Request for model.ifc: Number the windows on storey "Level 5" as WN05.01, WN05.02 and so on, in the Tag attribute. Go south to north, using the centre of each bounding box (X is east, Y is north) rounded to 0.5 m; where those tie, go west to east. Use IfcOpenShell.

First a look at what the model holds.

```python
import ifcopenshell
import ifcopenshell.util.element
import ifcopenshell.util.placement

model = ifcopenshell.open("model.ifc")
print(model.schema)
storey = next(s for s in model.by_type("IfcBuildingStorey") if s.Name == "Level 5")
windows = [e for e in ifcopenshell.util.element.get_decomposition(storey) if e.is_a("IfcWindow")]
for e in sorted(windows, key=lambda e: e.id()):
    origin = ifcopenshell.util.placement.get_local_placement(e.ObjectPlacement)[:3, 3]
    print(e.id(), e.Tag, e.Name, origin.round(2) + 0.0, sep=" | ")
```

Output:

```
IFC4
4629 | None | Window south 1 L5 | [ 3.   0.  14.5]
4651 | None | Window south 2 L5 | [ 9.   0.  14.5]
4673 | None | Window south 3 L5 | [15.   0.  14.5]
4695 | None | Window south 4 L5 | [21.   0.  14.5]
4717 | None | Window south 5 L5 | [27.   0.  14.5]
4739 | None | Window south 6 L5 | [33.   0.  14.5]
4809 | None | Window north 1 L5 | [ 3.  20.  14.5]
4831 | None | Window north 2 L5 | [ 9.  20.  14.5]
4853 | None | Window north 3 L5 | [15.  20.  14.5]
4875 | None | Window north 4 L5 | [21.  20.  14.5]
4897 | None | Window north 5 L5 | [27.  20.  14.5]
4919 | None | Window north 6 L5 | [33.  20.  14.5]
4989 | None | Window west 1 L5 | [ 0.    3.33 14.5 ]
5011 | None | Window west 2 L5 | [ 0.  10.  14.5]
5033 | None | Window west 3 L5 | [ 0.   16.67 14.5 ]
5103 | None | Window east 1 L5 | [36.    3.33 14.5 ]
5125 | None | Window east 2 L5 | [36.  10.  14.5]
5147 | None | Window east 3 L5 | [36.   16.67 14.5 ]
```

```python
import ifcopenshell
import ifcopenshell.geom
import ifcopenshell.util.element
import ifcopenshell.util.shape

model = ifcopenshell.open("model.ifc")
settings = ifcopenshell.geom.settings()
settings.set("use-world-coords", True)


def centre(element):
    shape = ifcopenshell.geom.create_shape(settings, element)
    return ifcopenshell.util.shape.get_bbox_centroid(shape.geometry)


storey = next(s for s in model.by_type("IfcBuildingStorey") if s.Name == "Level 5")
windows = [e for e in ifcopenshell.util.element.get_decomposition(storey) if e.is_a("IfcWindow")]

# Insertion points can sit at a corner or the storey origin, so sort by the geometry (in metres).
centres = {e: centre(e) for e in windows}
windows.sort(key=lambda e: (round(centres[e][1] / 0.5), centres[e][0]))

for i, e in enumerate(windows, start=1):
    number = f"WN05.{i:02d}"
    e.Tag = number
    print(e.id(), number)

model.write("model_edited.ifc")
```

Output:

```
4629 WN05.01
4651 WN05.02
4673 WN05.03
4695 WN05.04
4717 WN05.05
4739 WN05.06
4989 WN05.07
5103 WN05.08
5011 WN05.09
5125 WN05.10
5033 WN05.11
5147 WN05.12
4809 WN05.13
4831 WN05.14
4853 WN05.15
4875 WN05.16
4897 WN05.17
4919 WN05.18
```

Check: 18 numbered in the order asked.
